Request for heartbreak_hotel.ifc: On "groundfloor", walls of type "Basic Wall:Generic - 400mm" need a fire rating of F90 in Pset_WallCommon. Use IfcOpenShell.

First a look at what the model holds.

```python
import ifcopenshell
import ifcopenshell.util.element

model = ifcopenshell.open("heartbreak_hotel.ifc")
print(model.schema)
storey = next(s for s in model.by_type("IfcBuildingStorey") if s.Name == "groundfloor")
walls = [e for e in ifcopenshell.util.element.get_decomposition(storey) if e.is_a("IfcWall")]
seen = {}
for e in walls:
    element_type = ifcopenshell.util.element.get_type(e)
    key = (element_type.Name if element_type != e and element_type else None, ifcopenshell.util.element.get_pset(e, "Pset_WallCommon", "FireRating"))
    seen[key] = seen.get(key, 0) + 1
for (name, value), count in sorted(seen.items(), key=str):
    print(count, "x", name, "|", value)
```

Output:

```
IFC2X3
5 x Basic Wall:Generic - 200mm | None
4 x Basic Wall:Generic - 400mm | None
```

```python
import ifcopenshell
import ifcopenshell.api.pset
import ifcopenshell.util.element

model = ifcopenshell.open("heartbreak_hotel.ifc")

storey = next(s for s in model.by_type("IfcBuildingStorey") if s.Name == "groundfloor")
walls = [e for e in ifcopenshell.util.element.get_decomposition(storey) if e.is_a("IfcWall")]

count = 0
for e in walls:
    element_type = ifcopenshell.util.element.get_type(e)
    if element_type in (None, e) or element_type.Name != "Basic Wall:Generic - 400mm":
        continue
    # add_pset returns the element's existing set when there is one.
    pset = ifcopenshell.api.pset.add_pset(model, product=e, name="Pset_WallCommon")
    ifcopenshell.api.pset.edit_pset(model, pset=pset, properties={"FireRating": "F90"})
    count += 1

print(count, "walls updated")

model.write("heartbreak_hotel_v2.ifc")
```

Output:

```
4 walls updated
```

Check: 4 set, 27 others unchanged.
